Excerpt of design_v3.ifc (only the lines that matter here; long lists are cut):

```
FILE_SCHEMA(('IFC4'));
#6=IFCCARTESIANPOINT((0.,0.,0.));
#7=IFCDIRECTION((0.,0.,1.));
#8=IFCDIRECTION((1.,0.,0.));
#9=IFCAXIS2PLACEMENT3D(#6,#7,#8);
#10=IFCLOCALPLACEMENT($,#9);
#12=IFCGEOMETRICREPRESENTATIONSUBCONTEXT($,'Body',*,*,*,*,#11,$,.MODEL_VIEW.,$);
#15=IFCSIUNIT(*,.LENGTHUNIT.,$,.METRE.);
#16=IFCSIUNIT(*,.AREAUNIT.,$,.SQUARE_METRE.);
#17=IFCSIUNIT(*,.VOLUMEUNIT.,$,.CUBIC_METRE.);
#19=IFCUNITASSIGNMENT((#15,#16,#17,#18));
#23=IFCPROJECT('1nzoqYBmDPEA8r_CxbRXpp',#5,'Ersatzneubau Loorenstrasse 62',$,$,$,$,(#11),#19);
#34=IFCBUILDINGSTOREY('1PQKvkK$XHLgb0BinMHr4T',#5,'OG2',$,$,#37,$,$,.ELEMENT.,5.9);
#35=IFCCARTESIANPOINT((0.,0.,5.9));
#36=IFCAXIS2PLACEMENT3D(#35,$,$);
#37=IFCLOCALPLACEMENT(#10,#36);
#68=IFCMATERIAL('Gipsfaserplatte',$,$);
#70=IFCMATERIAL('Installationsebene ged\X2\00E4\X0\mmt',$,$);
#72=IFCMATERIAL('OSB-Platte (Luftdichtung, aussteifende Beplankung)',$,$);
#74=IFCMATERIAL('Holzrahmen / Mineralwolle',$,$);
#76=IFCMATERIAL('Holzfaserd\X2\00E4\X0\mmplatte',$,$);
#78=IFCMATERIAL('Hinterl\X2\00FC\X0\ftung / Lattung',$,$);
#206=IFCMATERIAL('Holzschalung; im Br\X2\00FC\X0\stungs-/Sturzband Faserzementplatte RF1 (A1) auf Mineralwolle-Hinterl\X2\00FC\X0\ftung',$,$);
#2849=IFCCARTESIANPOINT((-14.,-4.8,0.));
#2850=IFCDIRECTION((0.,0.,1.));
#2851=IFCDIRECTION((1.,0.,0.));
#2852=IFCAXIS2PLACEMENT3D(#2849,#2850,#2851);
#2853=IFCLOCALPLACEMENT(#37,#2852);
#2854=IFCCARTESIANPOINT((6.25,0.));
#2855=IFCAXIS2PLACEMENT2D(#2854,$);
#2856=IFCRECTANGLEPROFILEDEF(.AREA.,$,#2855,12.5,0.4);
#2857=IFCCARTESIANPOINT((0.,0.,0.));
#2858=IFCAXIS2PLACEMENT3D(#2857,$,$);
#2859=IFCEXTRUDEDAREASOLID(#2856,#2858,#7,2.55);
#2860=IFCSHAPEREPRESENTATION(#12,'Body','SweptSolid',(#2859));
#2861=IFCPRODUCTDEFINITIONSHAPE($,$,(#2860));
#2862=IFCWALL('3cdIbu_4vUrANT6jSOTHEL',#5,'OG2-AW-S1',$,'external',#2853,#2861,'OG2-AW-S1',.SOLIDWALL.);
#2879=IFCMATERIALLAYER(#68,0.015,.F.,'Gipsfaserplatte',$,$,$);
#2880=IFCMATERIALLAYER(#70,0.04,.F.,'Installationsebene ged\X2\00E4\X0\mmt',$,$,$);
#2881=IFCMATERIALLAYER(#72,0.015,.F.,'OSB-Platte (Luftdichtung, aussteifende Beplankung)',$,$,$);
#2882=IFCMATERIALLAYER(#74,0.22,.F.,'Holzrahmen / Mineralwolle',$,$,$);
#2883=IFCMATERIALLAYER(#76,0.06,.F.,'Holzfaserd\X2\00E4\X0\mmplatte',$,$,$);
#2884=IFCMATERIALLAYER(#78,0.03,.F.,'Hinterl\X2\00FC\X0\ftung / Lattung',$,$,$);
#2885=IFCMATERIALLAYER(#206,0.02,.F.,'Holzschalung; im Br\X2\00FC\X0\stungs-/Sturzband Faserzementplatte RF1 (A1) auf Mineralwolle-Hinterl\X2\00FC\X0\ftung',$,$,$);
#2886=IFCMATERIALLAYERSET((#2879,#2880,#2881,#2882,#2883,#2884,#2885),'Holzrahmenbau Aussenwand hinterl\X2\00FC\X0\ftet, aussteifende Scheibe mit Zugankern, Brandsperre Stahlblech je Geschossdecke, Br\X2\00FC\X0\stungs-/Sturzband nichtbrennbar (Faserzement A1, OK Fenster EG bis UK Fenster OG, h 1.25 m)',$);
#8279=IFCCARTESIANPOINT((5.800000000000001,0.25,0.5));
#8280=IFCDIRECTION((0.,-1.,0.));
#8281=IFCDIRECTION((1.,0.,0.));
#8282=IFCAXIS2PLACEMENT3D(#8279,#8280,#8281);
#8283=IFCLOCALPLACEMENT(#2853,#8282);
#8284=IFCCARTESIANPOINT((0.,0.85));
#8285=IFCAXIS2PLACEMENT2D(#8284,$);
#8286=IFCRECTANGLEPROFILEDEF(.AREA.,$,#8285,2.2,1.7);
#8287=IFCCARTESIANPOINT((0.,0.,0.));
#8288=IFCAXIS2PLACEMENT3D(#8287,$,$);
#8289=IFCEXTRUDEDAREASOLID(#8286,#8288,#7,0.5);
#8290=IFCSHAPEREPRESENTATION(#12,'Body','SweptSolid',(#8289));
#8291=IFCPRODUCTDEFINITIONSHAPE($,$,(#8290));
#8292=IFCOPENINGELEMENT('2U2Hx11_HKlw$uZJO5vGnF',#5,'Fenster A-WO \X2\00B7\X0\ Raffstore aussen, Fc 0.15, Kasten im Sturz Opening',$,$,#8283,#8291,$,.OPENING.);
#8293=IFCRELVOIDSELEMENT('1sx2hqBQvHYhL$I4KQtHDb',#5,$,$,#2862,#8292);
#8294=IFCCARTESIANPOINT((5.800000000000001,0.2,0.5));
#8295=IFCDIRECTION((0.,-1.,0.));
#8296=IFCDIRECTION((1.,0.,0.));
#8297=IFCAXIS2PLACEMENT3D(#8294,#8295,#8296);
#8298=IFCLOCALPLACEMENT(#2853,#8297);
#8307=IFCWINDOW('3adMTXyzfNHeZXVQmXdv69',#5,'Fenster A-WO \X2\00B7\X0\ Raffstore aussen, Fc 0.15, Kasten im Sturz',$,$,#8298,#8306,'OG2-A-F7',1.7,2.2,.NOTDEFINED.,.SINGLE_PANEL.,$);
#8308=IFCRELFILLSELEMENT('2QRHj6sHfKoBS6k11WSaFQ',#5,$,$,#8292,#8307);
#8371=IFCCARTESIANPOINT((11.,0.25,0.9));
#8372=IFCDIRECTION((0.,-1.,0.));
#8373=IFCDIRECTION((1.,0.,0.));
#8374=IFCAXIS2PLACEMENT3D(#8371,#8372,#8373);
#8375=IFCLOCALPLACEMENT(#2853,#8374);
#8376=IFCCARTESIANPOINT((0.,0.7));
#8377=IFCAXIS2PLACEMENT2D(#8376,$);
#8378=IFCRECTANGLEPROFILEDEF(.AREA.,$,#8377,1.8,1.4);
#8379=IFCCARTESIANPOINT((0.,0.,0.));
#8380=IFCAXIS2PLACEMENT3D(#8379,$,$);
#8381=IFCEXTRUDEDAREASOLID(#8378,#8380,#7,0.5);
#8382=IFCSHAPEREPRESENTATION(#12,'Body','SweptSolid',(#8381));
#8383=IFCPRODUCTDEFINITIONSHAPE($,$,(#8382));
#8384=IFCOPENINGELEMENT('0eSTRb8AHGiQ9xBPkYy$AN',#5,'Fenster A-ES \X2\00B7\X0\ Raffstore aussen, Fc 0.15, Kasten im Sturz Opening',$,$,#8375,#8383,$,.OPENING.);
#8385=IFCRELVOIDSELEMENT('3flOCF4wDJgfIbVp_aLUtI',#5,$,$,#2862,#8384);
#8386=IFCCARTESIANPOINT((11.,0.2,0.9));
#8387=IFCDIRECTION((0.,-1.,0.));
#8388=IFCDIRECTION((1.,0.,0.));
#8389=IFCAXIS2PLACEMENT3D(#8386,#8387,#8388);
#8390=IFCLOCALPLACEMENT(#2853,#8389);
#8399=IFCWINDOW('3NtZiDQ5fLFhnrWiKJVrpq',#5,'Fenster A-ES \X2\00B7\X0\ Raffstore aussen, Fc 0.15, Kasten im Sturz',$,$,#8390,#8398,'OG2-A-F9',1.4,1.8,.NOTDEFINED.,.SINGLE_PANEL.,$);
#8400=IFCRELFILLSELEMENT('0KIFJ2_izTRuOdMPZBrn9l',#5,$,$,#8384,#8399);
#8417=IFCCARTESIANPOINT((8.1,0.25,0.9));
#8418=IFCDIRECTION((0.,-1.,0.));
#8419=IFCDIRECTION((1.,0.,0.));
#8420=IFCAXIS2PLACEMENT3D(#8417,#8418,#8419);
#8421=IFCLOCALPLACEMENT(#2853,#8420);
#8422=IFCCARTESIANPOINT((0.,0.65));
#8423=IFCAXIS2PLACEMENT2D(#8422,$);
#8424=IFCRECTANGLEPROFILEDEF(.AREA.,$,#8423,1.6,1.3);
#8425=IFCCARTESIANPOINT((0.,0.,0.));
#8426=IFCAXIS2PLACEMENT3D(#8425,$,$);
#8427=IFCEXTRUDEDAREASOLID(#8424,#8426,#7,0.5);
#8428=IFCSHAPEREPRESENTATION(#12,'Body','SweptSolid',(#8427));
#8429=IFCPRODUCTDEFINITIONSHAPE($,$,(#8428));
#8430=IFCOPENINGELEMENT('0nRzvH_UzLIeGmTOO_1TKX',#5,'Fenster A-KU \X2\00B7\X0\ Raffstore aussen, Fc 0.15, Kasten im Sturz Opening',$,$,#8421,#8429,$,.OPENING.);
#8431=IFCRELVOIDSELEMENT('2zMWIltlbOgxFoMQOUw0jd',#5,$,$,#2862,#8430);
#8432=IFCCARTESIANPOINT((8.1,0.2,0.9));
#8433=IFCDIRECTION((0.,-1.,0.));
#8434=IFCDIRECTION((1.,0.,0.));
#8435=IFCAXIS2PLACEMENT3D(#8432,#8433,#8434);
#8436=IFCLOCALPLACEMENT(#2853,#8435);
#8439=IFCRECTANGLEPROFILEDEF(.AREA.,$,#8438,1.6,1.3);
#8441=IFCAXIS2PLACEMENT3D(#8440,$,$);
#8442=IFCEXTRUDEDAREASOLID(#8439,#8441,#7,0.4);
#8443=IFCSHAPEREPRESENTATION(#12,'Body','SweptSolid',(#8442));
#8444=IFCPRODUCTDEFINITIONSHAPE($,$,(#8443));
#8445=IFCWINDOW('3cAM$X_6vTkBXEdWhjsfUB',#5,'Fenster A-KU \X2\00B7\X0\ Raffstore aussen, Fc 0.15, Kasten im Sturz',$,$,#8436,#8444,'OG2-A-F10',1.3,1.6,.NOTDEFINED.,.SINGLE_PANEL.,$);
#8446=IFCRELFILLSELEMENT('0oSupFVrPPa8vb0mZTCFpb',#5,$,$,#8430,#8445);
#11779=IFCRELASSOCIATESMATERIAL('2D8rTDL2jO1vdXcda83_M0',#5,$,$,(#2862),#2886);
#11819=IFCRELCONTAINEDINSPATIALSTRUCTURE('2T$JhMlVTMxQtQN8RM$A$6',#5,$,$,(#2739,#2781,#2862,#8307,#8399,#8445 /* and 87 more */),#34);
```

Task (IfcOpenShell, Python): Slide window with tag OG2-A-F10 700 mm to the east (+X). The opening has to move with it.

```python
import ifcopenshell
import ifcopenshell.api.geometry
import ifcopenshell.util.placement

model = ifcopenshell.open("design_v3.ifc")

window = model.by_id(8445)
opening = window.FillsVoids[0].RelatingOpeningElement
wall = opening.VoidsElements[0].RelatingBuildingElement

wall_matrix = ifcopenshell.util.placement.get_local_placement(wall.ObjectPlacement)
shift = wall_matrix[:3, 0] * 0.7
before = ifcopenshell.util.placement.get_local_placement(window.ObjectPlacement)[:3, 3].copy()

# The window is not placed relative to its opening, so move both.
for product in (opening, window):
    matrix = ifcopenshell.util.placement.get_local_placement(product.ObjectPlacement)
    matrix[:3, 3] += shift
    ifcopenshell.api.geometry.edit_object_placement(model, product=product, matrix=matrix, is_si=False)

after = ifcopenshell.util.placement.get_local_placement(window.ObjectPlacement)[:3, 3]
print("window moved by", (after - before).round(3) + 0.0)

model.write("design_v3_v2.ifc")
```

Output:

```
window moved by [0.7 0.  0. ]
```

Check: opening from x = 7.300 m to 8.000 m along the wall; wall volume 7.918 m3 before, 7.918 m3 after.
